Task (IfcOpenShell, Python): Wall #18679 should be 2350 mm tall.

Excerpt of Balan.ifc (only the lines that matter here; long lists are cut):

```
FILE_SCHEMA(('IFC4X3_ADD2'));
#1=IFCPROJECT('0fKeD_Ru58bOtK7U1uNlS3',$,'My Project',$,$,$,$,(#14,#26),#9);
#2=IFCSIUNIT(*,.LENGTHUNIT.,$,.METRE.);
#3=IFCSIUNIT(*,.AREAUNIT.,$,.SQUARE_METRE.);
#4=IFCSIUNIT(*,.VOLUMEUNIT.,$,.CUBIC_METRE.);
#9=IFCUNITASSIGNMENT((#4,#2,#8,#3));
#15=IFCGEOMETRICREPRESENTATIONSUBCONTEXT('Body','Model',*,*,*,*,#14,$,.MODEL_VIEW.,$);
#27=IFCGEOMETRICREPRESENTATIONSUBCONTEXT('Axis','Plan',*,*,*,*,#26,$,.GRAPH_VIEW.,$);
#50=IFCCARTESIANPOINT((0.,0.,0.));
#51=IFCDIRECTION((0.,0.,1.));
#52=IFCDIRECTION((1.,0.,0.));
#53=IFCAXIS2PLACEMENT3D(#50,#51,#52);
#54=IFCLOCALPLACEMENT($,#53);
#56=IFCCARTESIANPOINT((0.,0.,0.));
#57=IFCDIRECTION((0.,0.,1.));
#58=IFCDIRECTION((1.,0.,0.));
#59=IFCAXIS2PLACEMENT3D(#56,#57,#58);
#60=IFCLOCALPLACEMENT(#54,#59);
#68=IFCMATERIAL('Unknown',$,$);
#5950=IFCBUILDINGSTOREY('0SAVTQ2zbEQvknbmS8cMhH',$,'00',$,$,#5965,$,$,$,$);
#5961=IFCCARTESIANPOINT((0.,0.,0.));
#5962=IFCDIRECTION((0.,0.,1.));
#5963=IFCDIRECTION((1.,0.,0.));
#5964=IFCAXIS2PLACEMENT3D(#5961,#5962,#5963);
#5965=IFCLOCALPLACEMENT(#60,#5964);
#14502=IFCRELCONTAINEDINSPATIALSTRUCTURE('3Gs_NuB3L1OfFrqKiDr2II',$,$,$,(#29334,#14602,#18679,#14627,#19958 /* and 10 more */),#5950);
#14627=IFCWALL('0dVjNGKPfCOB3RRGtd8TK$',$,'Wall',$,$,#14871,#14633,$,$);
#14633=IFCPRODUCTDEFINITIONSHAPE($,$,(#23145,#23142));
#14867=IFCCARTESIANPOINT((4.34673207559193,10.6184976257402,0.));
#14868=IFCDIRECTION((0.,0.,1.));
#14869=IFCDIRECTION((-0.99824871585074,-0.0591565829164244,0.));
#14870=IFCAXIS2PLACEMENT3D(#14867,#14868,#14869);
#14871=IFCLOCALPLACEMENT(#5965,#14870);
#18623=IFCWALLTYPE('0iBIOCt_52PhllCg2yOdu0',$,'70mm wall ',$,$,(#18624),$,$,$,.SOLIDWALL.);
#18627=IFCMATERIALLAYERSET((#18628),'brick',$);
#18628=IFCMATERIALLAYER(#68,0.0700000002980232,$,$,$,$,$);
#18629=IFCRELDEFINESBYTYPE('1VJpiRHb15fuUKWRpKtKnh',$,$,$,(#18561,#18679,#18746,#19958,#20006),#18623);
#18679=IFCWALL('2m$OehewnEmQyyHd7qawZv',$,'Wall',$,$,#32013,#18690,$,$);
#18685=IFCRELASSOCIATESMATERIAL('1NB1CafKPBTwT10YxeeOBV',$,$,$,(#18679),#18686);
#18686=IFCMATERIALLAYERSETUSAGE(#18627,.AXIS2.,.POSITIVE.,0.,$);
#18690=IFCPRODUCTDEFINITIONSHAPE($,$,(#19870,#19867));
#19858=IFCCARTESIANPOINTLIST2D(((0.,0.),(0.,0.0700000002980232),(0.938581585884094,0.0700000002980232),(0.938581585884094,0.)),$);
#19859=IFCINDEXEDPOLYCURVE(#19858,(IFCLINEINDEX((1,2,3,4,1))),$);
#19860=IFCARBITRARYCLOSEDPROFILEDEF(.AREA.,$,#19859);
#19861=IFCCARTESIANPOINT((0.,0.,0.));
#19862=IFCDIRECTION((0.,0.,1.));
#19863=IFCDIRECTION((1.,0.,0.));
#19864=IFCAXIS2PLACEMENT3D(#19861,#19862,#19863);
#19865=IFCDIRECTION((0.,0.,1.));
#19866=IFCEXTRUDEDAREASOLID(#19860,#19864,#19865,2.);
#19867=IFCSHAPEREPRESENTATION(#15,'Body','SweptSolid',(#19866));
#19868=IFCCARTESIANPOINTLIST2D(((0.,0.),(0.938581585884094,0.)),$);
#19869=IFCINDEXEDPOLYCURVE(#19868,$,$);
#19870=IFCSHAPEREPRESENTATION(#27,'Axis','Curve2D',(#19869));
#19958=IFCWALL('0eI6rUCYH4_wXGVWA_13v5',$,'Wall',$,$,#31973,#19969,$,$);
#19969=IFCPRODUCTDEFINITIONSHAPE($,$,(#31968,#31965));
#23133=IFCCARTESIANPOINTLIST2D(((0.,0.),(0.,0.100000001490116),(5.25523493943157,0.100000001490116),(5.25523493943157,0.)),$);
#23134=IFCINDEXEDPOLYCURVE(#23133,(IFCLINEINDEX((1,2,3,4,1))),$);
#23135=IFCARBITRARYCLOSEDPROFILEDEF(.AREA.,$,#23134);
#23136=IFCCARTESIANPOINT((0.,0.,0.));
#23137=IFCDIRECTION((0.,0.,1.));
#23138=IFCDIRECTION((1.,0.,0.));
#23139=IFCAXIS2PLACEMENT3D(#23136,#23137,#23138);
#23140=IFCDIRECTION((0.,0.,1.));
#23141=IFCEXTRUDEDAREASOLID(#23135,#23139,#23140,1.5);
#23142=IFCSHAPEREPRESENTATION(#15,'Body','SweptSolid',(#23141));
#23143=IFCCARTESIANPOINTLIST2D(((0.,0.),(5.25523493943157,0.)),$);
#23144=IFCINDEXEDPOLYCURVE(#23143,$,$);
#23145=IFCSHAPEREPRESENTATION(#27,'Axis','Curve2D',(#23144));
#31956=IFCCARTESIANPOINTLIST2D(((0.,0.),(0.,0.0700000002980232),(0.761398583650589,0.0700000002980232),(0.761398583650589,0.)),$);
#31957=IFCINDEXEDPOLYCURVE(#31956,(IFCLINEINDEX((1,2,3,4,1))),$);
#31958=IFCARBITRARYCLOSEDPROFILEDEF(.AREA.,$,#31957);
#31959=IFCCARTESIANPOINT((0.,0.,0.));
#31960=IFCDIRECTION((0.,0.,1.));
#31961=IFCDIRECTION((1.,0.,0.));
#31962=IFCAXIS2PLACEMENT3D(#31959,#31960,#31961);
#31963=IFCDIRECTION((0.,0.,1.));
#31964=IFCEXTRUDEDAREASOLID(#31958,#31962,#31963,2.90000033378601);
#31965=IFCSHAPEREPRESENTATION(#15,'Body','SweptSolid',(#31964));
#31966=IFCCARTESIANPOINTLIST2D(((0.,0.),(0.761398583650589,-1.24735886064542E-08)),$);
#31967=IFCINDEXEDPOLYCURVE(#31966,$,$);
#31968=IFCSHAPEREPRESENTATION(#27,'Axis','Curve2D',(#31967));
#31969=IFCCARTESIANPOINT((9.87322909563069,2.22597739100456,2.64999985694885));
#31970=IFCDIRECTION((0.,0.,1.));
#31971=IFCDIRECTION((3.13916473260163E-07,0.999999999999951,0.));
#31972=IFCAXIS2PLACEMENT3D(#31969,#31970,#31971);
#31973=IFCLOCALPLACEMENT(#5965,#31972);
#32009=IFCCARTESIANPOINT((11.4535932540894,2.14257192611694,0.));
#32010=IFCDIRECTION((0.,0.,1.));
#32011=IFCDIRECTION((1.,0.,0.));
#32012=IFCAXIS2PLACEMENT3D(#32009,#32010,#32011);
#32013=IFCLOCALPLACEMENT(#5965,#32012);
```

```python
import ifcopenshell
import ifcopenshell.geom
import ifcopenshell.util.representation
import ifcopenshell.util.shape

model = ifcopenshell.open("Balan.ifc")
settings = ifcopenshell.geom.settings()


def volume(element):
    """Net volume in cubic metres, openings subtracted."""
    shape = ifcopenshell.geom.create_shape(settings, element)
    return ifcopenshell.util.shape.get_volume(shape.geometry)


wall = model.by_guid("2m$OehewnEmQyyHd7qawZv")
before = volume(wall)

body = ifcopenshell.util.representation.get_representation(wall, "Model", "Body")
solid = body.Items[0]
old_height = solid.Depth
solid.Depth = 2.35
after = volume(wall)

print(f"height {old_height:g} -> {solid.Depth:g}, volume {before:.3f} -> {after:.3f} m3")

model.write("Balan_rev.ifc")
```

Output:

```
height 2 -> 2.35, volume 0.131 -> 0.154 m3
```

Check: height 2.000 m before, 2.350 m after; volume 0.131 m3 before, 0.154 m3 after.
